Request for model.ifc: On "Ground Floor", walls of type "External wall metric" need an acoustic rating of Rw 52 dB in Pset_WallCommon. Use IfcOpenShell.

First a look at what the model holds.

```python
import ifcopenshell
import ifcopenshell.util.element

model = ifcopenshell.open("model.ifc")
print(model.schema)
storey = next(s for s in model.by_type("IfcBuildingStorey") if s.Name == "Ground Floor")
walls = [e for e in ifcopenshell.util.element.get_decomposition(storey) if e.is_a("IfcWall")]
seen = {}
for e in walls:
    element_type = ifcopenshell.util.element.get_type(e)
    key = (element_type.Name if element_type != e and element_type else None, ifcopenshell.util.element.get_pset(e, "Pset_WallCommon", "AcousticRating"))
    seen[key] = seen.get(key, 0) + 1
for (name, value), count in sorted(seen.items(), key=str):
    print(count, "x", name, "|", value)
```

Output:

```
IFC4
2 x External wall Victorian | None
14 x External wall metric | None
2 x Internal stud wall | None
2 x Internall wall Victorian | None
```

```python
import ifcopenshell
import ifcopenshell.api.pset
import ifcopenshell.util.element

model = ifcopenshell.open("model.ifc")

storey = next(s for s in model.by_type("IfcBuildingStorey") if s.Name == "Ground Floor")
walls = [e for e in ifcopenshell.util.element.get_decomposition(storey) if e.is_a("IfcWall")]

count = 0
for e in walls:
    element_type = ifcopenshell.util.element.get_type(e)
    if element_type in (None, e) or element_type.Name != "External wall metric":
        continue
    # add_pset returns the element's existing set when there is one.
    pset = ifcopenshell.api.pset.add_pset(model, product=e, name="Pset_WallCommon")
    ifcopenshell.api.pset.edit_pset(model, pset=pset, properties={"AcousticRating": "Rw 52 dB"})
    count += 1

print(count, "walls updated")

model.write("model_rev.ifc")
```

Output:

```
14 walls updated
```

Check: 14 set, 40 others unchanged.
